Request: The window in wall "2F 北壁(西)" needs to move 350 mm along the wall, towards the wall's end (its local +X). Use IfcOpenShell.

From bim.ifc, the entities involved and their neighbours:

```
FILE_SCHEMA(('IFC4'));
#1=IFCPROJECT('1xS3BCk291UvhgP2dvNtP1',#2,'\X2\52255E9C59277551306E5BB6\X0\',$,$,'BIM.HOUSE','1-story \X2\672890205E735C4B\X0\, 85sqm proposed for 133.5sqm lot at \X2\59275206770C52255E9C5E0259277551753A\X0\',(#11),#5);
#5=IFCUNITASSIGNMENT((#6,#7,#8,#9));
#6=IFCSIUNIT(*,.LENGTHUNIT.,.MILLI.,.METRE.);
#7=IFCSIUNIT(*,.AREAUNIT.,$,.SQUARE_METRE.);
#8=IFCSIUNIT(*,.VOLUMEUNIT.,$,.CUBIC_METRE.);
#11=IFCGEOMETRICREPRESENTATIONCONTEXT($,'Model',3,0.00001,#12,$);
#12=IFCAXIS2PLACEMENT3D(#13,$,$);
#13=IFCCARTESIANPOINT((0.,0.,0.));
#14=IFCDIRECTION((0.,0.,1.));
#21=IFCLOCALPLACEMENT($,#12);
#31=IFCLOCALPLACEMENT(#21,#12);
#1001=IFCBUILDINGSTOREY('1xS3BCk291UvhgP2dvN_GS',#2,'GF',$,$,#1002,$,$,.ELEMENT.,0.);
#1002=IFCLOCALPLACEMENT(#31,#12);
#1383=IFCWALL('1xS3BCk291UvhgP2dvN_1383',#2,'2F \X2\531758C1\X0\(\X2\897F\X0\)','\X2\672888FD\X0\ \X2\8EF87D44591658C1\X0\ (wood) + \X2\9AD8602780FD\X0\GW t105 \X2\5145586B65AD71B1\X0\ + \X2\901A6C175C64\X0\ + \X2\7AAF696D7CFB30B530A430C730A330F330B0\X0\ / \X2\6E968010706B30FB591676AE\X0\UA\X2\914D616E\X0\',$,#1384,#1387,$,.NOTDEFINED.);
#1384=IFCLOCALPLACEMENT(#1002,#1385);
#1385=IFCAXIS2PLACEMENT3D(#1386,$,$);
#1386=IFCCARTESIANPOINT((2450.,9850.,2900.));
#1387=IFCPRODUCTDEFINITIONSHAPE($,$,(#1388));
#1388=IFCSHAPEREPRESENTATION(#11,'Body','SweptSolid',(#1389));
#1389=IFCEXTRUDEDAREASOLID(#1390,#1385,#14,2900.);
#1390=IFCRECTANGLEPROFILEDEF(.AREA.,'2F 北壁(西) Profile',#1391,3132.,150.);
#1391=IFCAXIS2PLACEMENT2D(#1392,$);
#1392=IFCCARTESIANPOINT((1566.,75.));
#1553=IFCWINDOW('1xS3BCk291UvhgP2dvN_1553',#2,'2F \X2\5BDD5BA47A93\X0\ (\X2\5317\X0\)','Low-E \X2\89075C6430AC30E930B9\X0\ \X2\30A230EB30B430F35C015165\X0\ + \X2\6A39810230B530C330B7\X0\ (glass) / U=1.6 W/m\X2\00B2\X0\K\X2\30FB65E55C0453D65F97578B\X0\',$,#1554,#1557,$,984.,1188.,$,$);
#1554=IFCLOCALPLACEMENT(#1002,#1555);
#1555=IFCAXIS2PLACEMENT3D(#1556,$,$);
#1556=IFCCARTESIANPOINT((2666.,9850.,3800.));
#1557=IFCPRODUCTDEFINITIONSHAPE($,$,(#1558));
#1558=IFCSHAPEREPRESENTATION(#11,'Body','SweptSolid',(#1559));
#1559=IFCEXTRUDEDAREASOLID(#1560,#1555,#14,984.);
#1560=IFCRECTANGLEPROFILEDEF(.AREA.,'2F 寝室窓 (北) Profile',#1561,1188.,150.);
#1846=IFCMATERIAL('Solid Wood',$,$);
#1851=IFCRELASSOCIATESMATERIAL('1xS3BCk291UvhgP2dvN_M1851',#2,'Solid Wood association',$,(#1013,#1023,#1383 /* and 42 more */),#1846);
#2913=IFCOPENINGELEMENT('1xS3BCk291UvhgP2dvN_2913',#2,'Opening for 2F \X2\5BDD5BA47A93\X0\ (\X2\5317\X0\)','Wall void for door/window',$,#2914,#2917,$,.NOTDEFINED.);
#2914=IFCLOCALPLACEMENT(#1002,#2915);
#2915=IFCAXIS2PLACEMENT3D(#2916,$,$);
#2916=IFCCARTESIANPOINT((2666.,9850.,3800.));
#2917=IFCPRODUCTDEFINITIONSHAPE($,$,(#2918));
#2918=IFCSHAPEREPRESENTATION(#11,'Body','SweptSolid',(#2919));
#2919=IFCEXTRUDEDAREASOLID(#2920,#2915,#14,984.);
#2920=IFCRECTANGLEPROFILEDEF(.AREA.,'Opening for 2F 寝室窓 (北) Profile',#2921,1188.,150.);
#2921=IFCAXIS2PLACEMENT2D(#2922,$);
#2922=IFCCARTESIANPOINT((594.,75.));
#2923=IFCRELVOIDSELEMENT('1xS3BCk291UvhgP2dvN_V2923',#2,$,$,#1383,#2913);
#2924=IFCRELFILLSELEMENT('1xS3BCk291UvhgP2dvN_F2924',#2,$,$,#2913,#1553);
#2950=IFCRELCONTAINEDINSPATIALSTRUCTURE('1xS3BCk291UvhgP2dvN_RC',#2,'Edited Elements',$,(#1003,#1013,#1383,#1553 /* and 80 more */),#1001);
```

```python
import ifcopenshell
import ifcopenshell.api.geometry
import ifcopenshell.util.placement
import ifcopenshell.util.unit

model = ifcopenshell.open("bim.ifc")
unit_scale = ifcopenshell.util.unit.calculate_unit_scale(model)

window = model.by_guid("1xS3BCk291UvhgP2dvN_1553")
opening = window.FillsVoids[0].RelatingOpeningElement
wall = opening.VoidsElements[0].RelatingBuildingElement

wall_matrix = ifcopenshell.util.placement.get_local_placement(wall.ObjectPlacement)
shift = wall_matrix[:3, 0] * 0.35 / unit_scale
before = ifcopenshell.util.placement.get_local_placement(window.ObjectPlacement)[:3, 3].copy()

# The window is not placed relative to its opening, so move both.
for product in (opening, window):
    matrix = ifcopenshell.util.placement.get_local_placement(product.ObjectPlacement)
    matrix[:3, 3] += shift
    ifcopenshell.api.geometry.edit_object_placement(model, product=product, matrix=matrix, is_si=False)

after = ifcopenshell.util.placement.get_local_placement(window.ObjectPlacement)[:3, 3]
print("window moved by", (after - before).round(3) + 0.0)

model.write("bim_edited.ifc")
```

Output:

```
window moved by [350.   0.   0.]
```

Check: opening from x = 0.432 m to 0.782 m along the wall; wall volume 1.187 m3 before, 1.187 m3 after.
